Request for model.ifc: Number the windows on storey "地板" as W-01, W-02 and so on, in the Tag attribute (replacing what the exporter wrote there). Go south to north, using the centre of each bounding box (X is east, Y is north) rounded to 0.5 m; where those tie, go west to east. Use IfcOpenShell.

First a look at what the model holds.

```python
import ifcopenshell
import ifcopenshell.util.element
import ifcopenshell.util.placement

model = ifcopenshell.open("model.ifc")
print(model.schema)
storey = next(s for s in model.by_type("IfcBuildingStorey") if s.Name == "地板")
windows = [e for e in ifcopenshell.util.element.get_decomposition(storey) if e.is_a("IfcWindow")]
for e in sorted(windows, key=lambda e: e.id()):
    origin = ifcopenshell.util.placement.get_local_placement(e.ObjectPlacement)[:3, 3]
    print(e.id(), e.Tag, e.Name, origin.round(2) + 0.0, sep=" | ")
```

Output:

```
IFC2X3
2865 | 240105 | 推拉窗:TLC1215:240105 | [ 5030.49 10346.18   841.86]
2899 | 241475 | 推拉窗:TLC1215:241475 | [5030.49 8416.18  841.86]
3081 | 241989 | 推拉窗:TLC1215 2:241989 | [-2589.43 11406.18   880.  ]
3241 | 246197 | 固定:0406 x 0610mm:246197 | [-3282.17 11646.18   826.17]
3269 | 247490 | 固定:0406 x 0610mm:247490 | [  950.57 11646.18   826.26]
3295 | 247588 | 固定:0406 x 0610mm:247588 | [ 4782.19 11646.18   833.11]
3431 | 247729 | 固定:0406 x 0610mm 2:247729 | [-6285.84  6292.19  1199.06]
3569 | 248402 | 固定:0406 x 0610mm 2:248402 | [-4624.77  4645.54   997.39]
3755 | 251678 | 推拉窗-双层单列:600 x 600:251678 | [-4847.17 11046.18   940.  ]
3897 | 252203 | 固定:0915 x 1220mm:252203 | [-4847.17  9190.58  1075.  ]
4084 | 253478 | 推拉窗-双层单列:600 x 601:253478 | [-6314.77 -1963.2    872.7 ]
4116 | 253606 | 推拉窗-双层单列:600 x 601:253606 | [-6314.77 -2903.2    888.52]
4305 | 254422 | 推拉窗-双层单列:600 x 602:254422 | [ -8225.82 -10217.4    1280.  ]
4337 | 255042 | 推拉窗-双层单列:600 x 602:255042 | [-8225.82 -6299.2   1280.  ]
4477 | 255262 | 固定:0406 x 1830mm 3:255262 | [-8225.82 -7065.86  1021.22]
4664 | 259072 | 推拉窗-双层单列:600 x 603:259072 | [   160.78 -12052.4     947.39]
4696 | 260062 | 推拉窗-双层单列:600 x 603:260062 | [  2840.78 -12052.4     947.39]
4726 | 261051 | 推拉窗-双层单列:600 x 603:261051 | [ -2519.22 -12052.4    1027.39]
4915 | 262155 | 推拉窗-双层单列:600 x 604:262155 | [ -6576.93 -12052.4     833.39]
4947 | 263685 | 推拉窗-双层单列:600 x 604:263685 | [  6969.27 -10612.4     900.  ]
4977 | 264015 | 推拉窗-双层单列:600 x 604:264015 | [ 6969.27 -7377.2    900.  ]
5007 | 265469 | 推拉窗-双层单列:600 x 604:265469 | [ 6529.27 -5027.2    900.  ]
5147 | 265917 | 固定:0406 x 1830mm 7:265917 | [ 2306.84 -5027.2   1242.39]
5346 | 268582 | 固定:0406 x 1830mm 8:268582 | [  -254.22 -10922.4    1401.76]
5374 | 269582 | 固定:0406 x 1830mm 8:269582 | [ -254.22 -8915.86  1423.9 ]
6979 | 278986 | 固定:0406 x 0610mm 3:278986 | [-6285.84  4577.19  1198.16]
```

```python
import ifcopenshell
import ifcopenshell.geom
import ifcopenshell.util.element
import ifcopenshell.util.shape

model = ifcopenshell.open("model.ifc")
settings = ifcopenshell.geom.settings()
settings.set("use-world-coords", True)


def centre(element):
    shape = ifcopenshell.geom.create_shape(settings, element)
    return ifcopenshell.util.shape.get_bbox_centroid(shape.geometry)


storey = next(s for s in model.by_type("IfcBuildingStorey") if s.Name == "地板")
windows = [e for e in ifcopenshell.util.element.get_decomposition(storey) if e.is_a("IfcWindow")]

# Insertion points can sit at a corner or the storey origin, so sort by the geometry (in metres).
centres = {e: centre(e) for e in windows}
windows.sort(key=lambda e: (round(centres[e][1] / 0.5), centres[e][0]))

for i, e in enumerate(windows, start=1):
    number = f"W-{i:02d}"
    e.Tag = number
    print(e.id(), number)

model.write("model_edited.ifc")
```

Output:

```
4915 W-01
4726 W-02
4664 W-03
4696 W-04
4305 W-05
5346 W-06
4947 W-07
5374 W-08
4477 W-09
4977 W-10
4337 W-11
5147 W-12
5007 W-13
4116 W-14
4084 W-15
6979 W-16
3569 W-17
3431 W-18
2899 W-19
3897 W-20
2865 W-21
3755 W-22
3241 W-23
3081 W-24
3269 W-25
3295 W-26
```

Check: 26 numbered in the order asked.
